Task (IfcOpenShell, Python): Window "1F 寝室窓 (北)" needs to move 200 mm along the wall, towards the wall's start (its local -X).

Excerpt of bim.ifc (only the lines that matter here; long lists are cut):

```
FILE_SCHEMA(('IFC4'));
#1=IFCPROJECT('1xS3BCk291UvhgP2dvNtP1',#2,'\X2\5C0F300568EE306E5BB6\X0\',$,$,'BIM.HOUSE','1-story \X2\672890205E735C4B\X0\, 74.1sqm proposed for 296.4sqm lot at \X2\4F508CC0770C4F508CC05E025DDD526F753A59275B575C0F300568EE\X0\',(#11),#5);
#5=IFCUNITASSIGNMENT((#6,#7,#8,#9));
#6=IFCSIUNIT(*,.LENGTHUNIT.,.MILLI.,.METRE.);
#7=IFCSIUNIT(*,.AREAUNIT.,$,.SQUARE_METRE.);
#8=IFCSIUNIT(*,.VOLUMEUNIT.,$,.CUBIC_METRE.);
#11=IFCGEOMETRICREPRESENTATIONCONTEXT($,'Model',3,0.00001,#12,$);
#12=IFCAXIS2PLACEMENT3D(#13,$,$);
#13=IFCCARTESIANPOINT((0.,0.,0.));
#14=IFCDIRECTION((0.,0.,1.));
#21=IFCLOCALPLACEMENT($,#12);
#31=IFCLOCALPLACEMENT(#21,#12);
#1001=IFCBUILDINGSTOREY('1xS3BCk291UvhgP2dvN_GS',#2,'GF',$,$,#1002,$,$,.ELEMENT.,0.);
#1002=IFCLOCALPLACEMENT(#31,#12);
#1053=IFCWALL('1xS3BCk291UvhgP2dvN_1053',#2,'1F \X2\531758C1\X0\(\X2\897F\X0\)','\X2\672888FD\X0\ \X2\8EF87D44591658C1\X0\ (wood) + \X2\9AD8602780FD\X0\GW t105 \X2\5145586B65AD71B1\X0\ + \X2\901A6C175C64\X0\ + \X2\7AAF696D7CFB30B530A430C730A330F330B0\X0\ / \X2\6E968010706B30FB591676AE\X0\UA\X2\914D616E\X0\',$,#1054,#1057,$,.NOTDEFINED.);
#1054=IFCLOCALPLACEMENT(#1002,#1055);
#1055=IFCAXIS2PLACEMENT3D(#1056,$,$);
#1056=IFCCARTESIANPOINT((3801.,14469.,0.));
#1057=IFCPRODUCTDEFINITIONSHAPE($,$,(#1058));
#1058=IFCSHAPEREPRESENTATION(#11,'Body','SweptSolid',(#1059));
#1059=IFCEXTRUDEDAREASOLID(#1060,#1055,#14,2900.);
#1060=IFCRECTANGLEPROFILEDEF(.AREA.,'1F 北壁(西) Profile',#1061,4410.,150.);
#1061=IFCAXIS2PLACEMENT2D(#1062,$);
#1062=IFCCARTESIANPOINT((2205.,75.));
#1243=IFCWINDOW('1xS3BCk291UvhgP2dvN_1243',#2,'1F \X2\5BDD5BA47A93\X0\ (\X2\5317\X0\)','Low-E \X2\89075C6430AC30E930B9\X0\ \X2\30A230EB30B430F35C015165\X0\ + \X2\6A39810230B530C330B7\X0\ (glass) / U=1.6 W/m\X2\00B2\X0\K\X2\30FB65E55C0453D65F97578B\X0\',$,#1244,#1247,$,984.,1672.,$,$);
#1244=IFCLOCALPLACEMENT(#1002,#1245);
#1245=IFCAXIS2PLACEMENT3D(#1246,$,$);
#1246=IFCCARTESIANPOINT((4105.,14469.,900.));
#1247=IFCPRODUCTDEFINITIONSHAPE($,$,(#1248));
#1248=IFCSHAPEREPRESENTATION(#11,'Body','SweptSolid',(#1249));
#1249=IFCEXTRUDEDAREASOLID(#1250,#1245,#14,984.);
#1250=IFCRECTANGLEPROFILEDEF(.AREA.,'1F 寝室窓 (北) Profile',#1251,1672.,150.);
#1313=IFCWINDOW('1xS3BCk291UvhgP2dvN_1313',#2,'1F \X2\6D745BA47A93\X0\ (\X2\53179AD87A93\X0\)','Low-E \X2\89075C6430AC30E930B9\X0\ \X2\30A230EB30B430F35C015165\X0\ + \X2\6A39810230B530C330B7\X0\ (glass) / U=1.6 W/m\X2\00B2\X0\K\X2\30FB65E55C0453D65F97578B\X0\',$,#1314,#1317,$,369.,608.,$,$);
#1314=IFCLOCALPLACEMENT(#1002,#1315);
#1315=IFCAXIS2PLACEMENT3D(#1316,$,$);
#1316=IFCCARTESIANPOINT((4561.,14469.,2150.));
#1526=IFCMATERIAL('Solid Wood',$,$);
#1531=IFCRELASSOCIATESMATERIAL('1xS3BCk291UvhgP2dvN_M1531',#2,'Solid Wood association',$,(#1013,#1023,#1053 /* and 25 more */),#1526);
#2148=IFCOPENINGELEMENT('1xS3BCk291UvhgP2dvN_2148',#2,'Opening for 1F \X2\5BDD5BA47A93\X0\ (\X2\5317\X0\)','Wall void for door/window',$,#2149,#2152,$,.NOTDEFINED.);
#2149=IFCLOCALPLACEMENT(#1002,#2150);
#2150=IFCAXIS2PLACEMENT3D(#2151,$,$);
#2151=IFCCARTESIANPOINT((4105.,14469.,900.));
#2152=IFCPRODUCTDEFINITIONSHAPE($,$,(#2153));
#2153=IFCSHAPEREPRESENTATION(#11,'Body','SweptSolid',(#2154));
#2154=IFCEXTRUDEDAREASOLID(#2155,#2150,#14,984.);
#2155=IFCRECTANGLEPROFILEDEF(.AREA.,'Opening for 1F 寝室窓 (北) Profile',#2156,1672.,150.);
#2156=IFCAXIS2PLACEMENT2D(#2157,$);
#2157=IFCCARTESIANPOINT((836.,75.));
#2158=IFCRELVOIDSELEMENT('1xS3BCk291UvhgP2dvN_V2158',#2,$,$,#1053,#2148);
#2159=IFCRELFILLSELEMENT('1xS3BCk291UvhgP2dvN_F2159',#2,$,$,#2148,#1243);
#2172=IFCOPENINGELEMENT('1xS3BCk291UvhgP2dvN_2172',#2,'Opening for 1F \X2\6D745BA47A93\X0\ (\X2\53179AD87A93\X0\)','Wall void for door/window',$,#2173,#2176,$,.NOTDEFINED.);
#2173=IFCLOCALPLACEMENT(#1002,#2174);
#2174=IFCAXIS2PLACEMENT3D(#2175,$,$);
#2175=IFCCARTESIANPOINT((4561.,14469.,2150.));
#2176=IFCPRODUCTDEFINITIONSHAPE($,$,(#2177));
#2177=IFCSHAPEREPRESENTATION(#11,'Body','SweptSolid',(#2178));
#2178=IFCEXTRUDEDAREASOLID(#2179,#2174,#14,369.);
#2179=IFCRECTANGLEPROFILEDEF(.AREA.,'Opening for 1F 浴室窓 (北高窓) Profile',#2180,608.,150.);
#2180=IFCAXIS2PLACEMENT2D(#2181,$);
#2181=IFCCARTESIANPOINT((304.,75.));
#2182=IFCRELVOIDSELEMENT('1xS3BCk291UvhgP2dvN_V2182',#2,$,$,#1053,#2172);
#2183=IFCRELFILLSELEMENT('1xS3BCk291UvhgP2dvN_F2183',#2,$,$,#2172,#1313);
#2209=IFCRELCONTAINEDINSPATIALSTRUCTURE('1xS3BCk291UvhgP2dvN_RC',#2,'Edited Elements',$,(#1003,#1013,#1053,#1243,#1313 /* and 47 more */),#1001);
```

```python
import ifcopenshell
import ifcopenshell.api.geometry
import ifcopenshell.util.placement

model = ifcopenshell.open("bim.ifc")

window = model.by_id(1243)
opening = window.FillsVoids[0].RelatingOpeningElement
wall = opening.VoidsElements[0].RelatingBuildingElement

wall_matrix = ifcopenshell.util.placement.get_local_placement(wall.ObjectPlacement)
shift = wall_matrix[:3, 0] * -200.0
before = ifcopenshell.util.placement.get_local_placement(window.ObjectPlacement)[:3, 3].copy()

# The window is not placed relative to its opening, so move both.
for product in (opening, window):
    matrix = ifcopenshell.util.placement.get_local_placement(product.ObjectPlacement)
    matrix[:3, 3] += shift
    ifcopenshell.api.geometry.edit_object_placement(model, product=product, matrix=matrix, is_si=False)

after = ifcopenshell.util.placement.get_local_placement(window.ObjectPlacement)[:3, 3]
print("window moved by", (after - before).round(3) + 0.0)

model.write("bim_edited.ifc")
```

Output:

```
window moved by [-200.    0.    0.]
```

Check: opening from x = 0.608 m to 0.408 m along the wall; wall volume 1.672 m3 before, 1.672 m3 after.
